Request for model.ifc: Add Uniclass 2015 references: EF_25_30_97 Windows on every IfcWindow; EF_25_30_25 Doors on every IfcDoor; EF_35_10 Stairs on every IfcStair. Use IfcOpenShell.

First a look at what the model holds.

```python
import ifcopenshell

model = ifcopenshell.open("model.ifc")
print(model.schema)
print("classifications:", [c.Name for c in model.by_type("IfcClassification")])
for ifc_class in ("IfcDoor", "IfcRoof", "IfcStair", "IfcWall", "IfcWindow"):
    print(ifc_class, len(model.by_type(ifc_class)))
```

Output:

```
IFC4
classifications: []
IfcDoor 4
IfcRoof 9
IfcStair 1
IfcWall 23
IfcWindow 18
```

```python
import ifcopenshell
import ifcopenshell.api.classification

model = ifcopenshell.open("model.ifc")

system = ifcopenshell.api.classification.add_classification(model, classification="Uniclass 2015")

codes = {
    "IfcWindow": ("EF_25_30_97", "Windows"),
    "IfcDoor": ("EF_25_30_25", "Doors"),
    "IfcStair": ("EF_35_10", "Stairs"),
}
for ifc_class, (code, name) in codes.items():
    products = model.by_type(ifc_class)
    ifcopenshell.api.classification.add_reference(
        model, products=products, classification=system, identification=code, name=name
    )
    print(code, len(products))

model.write("model_rev.ifc")
```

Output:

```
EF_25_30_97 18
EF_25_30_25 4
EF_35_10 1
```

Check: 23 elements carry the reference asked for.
